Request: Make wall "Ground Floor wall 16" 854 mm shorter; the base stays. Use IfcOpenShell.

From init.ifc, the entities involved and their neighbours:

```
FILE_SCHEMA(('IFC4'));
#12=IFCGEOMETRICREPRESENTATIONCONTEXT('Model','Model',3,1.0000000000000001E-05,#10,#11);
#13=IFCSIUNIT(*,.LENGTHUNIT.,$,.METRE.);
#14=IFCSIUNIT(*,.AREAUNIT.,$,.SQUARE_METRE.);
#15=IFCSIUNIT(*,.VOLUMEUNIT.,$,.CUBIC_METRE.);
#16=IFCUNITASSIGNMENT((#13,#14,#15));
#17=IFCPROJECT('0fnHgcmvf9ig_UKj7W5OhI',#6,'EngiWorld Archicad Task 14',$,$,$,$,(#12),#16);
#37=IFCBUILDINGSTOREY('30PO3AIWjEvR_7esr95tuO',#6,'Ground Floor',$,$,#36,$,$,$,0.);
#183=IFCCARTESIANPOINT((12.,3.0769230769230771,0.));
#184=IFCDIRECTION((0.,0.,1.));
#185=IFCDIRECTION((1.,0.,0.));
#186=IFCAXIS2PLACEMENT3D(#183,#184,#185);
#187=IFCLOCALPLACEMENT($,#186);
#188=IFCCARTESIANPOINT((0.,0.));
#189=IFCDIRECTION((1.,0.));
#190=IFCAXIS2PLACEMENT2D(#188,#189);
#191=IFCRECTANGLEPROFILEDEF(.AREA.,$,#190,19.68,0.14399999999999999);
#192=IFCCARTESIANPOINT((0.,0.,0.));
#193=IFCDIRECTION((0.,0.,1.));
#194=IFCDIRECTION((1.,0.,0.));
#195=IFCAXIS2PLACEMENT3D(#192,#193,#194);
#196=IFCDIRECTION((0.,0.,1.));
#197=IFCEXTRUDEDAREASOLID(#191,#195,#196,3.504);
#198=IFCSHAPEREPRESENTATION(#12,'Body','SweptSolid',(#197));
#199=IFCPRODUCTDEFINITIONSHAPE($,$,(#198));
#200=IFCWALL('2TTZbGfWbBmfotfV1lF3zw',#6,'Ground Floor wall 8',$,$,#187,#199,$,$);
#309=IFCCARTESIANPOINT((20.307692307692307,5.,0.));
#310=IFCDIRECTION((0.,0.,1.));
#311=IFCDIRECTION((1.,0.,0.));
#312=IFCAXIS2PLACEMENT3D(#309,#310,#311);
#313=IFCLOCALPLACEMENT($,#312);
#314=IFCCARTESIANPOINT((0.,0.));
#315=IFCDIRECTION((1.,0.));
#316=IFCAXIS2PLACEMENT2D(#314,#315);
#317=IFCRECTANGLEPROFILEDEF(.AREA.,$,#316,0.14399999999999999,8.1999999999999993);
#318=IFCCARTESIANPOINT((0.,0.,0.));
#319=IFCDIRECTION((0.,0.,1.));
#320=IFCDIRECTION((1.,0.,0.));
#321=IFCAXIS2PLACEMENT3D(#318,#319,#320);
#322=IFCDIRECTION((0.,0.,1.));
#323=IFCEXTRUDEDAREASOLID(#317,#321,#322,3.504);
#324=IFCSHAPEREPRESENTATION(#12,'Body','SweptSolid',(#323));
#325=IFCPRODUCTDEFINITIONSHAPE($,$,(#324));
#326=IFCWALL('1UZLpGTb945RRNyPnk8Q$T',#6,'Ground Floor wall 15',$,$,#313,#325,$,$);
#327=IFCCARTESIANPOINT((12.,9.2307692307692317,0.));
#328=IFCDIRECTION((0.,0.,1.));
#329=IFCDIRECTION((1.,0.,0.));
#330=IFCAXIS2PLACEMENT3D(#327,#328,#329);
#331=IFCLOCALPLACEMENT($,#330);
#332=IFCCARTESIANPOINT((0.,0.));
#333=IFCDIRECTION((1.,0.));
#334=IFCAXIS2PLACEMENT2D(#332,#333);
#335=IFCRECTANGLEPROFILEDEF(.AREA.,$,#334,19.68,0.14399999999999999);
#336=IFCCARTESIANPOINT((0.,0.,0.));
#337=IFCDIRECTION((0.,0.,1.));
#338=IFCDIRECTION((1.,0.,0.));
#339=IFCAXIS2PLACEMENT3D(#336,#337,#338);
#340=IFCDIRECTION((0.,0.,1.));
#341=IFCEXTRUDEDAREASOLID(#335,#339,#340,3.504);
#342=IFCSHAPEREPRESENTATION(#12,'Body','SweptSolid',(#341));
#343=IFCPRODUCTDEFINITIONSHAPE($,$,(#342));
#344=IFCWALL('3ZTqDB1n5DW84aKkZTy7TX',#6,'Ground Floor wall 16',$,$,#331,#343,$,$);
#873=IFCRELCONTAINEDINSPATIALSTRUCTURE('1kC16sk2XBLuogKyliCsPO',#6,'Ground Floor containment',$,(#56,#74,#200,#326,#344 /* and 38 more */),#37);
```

```python
import ifcopenshell
import ifcopenshell.geom
import ifcopenshell.util.shape

model = ifcopenshell.open("init.ifc")
settings = ifcopenshell.geom.settings()


def volume(element):
    """Net volume in cubic metres, openings subtracted."""
    shape = ifcopenshell.geom.create_shape(settings, element)
    return ifcopenshell.util.shape.get_volume(shape.geometry)


wall = model.by_guid("3ZTqDB1n5DW84aKkZTy7TX")
before = volume(wall)

body = next(r for r in wall.Representation.Representations if r.RepresentationIdentifier == "Body")
solid = body.Items[0]
old_height = solid.Depth
solid.Depth -= 0.854
after = volume(wall)

print(f"height {old_height:g} -> {solid.Depth:g}, volume {before:.3f} -> {after:.3f} m3")

model.write("init_v2.ifc")
```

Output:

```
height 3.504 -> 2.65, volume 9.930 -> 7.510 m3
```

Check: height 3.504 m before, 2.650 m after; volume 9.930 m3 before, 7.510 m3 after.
